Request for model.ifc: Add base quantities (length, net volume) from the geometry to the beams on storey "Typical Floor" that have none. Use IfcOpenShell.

First a look at what the model holds.

```python
import ifcopenshell
import ifcopenshell.util.element
import ifcopenshell.util.unit

model = ifcopenshell.open("model.ifc")
print(model.schema)
for unit_type in ("LENGTHUNIT", "AREAUNIT", "VOLUMEUNIT"):
    print(unit_type, ifcopenshell.util.unit.calculate_unit_scale(model, unit_type))
storey = next(s for s in model.by_type("IfcBuildingStorey") if s.Name == "Typical Floor")
beams = [e for e in ifcopenshell.util.element.get_decomposition(storey) if e.is_a("IfcBeam")]
for e in sorted(beams, key=lambda e: e.id()):
    print(e.id(), e.is_a(), e.Name, list(ifcopenshell.util.element.get_psets(e, qtos_only=True)), sep=" | ")
```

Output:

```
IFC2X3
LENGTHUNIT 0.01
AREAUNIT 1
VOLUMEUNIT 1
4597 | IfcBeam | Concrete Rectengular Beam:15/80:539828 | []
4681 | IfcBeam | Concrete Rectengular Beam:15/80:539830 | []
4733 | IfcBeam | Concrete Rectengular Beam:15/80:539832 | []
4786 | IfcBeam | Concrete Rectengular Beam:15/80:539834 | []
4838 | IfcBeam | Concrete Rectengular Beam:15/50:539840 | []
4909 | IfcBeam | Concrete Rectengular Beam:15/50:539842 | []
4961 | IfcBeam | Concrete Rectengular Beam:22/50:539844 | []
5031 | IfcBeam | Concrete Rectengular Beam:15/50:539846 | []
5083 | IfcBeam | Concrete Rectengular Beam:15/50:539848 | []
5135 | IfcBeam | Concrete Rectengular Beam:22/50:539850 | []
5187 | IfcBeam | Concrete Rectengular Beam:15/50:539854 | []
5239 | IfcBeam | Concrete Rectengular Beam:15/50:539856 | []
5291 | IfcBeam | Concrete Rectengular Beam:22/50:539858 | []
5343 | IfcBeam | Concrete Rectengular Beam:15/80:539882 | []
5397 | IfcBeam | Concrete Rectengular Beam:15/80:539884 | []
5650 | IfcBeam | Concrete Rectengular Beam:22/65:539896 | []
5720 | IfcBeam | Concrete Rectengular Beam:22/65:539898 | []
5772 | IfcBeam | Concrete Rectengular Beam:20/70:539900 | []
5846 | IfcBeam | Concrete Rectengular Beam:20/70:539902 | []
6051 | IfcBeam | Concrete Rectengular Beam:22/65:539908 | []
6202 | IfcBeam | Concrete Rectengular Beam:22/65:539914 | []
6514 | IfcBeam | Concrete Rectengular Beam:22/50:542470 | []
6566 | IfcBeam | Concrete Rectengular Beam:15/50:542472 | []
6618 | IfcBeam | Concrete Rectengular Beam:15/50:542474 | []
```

```python
import ifcopenshell
import ifcopenshell.api.pset
import ifcopenshell.geom
import ifcopenshell.util.element
import ifcopenshell.util.shape
import ifcopenshell.util.unit

model = ifcopenshell.open("model.ifc")
unit_scale = ifcopenshell.util.unit.calculate_unit_scale(model)
volume_scale = ifcopenshell.util.unit.calculate_unit_scale(model, "VOLUMEUNIT")
settings = ifcopenshell.geom.settings()

storey = next(s for s in model.by_type("IfcBuildingStorey") if s.Name == "Typical Floor")
beams = [e for e in ifcopenshell.util.element.get_decomposition(storey) if e.is_a("IfcBeam")]

for e in sorted(beams, key=lambda e: e.id()):
    if ifcopenshell.util.element.get_psets(e, qtos_only=True, should_inherit=False):
        continue
    # Geometry comes back in metres, in the element's own axes.
    shape = ifcopenshell.geom.create_shape(settings, e)
    values = {
        "Length": ifcopenshell.util.shape.get_max_xyz(shape.geometry) / unit_scale,
        "NetVolume": ifcopenshell.util.shape.get_volume(shape.geometry) / volume_scale,
    }
    qto = ifcopenshell.api.pset.add_qto(model, product=e, name="BaseQuantities")
    ifcopenshell.api.pset.edit_qto(model, qto=qto, properties=values)
    print(e.id(), {k: round(v, 3) for k, v in values.items()})

model.write("model_rev.ifc")
```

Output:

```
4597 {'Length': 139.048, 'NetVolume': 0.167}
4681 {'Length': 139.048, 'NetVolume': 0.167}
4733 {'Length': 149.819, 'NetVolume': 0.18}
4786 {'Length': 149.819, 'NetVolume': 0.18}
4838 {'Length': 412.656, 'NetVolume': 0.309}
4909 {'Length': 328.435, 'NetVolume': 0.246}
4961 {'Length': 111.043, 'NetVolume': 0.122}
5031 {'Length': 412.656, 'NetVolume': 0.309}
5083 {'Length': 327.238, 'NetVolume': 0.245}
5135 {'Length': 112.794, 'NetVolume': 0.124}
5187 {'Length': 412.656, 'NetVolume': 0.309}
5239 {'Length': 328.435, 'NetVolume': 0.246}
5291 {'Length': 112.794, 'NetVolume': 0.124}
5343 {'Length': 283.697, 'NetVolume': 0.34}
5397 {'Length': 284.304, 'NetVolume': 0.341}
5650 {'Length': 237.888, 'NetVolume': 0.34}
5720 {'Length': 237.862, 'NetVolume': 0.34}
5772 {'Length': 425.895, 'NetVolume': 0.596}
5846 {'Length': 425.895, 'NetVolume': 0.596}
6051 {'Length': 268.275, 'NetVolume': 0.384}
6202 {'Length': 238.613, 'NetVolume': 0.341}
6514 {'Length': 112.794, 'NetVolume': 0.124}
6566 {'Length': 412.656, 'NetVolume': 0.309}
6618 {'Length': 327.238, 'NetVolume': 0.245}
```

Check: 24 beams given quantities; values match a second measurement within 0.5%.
